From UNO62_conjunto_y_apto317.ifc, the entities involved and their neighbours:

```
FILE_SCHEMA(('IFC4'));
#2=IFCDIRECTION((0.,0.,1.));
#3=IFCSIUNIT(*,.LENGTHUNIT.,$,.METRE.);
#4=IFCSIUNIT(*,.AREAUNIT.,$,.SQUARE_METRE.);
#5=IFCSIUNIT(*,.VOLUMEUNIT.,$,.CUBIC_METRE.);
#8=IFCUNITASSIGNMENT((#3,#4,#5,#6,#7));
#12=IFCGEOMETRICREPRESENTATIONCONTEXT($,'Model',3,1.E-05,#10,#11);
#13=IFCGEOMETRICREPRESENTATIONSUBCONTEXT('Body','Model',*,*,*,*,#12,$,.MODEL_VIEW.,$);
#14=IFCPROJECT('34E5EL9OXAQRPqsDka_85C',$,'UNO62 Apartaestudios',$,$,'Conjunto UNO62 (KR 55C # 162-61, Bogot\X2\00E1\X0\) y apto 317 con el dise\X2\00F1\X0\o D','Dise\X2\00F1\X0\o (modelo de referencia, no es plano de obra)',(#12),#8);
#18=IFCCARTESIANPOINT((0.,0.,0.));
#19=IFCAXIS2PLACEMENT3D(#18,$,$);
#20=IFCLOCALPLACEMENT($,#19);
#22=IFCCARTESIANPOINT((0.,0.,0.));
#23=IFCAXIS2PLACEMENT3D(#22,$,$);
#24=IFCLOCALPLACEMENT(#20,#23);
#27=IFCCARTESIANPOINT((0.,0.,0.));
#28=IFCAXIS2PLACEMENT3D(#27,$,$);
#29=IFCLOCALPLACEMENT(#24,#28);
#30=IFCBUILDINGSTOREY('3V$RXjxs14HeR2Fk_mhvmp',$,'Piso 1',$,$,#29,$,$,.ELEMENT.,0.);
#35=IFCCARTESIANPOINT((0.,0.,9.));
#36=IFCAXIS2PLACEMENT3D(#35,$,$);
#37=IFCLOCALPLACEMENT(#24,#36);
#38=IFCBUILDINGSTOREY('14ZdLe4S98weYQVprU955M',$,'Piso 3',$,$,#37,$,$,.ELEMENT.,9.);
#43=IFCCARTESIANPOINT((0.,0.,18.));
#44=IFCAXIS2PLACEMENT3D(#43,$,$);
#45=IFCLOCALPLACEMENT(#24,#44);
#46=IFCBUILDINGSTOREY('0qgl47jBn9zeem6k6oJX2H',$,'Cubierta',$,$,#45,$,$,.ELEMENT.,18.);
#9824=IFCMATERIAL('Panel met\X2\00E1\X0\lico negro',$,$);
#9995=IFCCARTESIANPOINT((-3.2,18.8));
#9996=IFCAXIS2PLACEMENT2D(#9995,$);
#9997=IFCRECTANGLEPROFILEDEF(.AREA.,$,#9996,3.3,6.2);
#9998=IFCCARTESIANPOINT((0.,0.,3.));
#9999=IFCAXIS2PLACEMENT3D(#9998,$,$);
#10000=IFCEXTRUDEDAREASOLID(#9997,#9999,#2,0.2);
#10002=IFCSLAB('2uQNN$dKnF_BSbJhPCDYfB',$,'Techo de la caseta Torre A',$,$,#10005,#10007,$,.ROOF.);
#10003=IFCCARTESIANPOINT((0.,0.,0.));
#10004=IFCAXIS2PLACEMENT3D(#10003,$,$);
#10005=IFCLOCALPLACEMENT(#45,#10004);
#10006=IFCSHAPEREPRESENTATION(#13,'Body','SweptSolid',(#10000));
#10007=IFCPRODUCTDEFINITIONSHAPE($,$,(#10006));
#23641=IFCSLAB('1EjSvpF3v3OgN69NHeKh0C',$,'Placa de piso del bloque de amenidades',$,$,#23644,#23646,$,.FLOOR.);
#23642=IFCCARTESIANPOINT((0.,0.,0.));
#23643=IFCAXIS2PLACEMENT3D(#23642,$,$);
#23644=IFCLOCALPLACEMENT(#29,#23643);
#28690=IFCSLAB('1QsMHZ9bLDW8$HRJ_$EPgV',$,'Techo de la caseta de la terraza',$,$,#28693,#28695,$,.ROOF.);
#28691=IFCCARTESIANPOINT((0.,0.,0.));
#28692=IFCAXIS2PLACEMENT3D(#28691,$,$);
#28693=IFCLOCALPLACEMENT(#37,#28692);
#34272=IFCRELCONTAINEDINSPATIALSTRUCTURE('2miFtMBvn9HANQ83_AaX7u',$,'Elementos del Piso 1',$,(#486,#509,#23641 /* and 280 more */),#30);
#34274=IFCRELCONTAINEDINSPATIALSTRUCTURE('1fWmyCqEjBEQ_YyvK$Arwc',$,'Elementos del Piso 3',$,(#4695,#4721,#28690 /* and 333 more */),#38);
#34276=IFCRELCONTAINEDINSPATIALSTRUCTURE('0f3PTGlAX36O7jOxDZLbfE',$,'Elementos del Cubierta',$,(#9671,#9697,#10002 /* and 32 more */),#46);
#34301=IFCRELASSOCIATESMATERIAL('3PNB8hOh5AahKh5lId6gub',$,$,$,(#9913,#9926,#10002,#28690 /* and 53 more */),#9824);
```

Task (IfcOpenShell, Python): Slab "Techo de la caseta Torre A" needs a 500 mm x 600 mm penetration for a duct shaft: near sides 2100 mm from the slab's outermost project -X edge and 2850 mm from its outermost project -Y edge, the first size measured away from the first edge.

```python
import numpy as np
import ifcopenshell
import ifcopenshell.api.feature
import ifcopenshell.api.geometry
import ifcopenshell.api.root
import ifcopenshell.geom
import ifcopenshell.util.placement
import ifcopenshell.util.representation
import ifcopenshell.util.shape
import ifcopenshell.util.unit

model = ifcopenshell.open("UNO62_conjunto_y_apto317.ifc")
unit_scale = ifcopenshell.util.unit.calculate_unit_scale(model)
settings = ifcopenshell.geom.settings()


def volume(element):
    """Net volume in cubic metres, openings subtracted."""
    shape = ifcopenshell.geom.create_shape(settings, element)
    return ifcopenshell.util.shape.get_volume(shape.geometry)


slab = model.by_guid("2uQNN$dKnF_BSbJhPCDYfB")
before = volume(slab)

# Extent in the slab's own axes, in metres. The edges named are its -X and -Y sides.
slab_shape = ifcopenshell.geom.create_shape(settings, slab)
vertices = ifcopenshell.util.shape.get_vertices(slab_shape.geometry)
x_min, y_min, bottom = vertices.min(axis=0)
top = vertices[:, 2].max()

opening = ifcopenshell.api.root.create_entity(model, ifc_class="IfcOpeningElement", name="Duct shaft opening", predefined_type="OPENING")
context = ifcopenshell.util.representation.get_context(model, "Model", "Body", "MODEL_VIEW")
width, depth = 0.5, 0.6
outline = [(0.0, 0.0), (width, 0.0), (width, depth), (0.0, depth), (0.0, 0.0)]
# Overshoot both faces by 50 mm so the cut is clean.
shape = ifcopenshell.api.geometry.add_slab_representation(
    model, context=context, depth=top - bottom + 0.1, polyline=outline
)
ifcopenshell.api.geometry.assign_representation(model, product=opening, representation=shape)

matrix = ifcopenshell.util.placement.get_local_placement(slab.ObjectPlacement)
matrix[:, 3] = matrix @ np.append(np.array([x_min + 2.1, y_min + 2.85, bottom - 0.05]) / unit_scale, 1.0)
ifcopenshell.api.geometry.edit_object_placement(model, product=opening, matrix=matrix, is_si=False)
ifcopenshell.api.feature.add_feature(model, feature=opening, element=slab)

after = volume(slab)

print(f"slab volume {before:.3f} -> {after:.3f} m3")

model.write("UNO62_conjunto_y_apto317-out.ifc")
```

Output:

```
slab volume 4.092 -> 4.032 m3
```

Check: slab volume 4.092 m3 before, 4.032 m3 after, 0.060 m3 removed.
